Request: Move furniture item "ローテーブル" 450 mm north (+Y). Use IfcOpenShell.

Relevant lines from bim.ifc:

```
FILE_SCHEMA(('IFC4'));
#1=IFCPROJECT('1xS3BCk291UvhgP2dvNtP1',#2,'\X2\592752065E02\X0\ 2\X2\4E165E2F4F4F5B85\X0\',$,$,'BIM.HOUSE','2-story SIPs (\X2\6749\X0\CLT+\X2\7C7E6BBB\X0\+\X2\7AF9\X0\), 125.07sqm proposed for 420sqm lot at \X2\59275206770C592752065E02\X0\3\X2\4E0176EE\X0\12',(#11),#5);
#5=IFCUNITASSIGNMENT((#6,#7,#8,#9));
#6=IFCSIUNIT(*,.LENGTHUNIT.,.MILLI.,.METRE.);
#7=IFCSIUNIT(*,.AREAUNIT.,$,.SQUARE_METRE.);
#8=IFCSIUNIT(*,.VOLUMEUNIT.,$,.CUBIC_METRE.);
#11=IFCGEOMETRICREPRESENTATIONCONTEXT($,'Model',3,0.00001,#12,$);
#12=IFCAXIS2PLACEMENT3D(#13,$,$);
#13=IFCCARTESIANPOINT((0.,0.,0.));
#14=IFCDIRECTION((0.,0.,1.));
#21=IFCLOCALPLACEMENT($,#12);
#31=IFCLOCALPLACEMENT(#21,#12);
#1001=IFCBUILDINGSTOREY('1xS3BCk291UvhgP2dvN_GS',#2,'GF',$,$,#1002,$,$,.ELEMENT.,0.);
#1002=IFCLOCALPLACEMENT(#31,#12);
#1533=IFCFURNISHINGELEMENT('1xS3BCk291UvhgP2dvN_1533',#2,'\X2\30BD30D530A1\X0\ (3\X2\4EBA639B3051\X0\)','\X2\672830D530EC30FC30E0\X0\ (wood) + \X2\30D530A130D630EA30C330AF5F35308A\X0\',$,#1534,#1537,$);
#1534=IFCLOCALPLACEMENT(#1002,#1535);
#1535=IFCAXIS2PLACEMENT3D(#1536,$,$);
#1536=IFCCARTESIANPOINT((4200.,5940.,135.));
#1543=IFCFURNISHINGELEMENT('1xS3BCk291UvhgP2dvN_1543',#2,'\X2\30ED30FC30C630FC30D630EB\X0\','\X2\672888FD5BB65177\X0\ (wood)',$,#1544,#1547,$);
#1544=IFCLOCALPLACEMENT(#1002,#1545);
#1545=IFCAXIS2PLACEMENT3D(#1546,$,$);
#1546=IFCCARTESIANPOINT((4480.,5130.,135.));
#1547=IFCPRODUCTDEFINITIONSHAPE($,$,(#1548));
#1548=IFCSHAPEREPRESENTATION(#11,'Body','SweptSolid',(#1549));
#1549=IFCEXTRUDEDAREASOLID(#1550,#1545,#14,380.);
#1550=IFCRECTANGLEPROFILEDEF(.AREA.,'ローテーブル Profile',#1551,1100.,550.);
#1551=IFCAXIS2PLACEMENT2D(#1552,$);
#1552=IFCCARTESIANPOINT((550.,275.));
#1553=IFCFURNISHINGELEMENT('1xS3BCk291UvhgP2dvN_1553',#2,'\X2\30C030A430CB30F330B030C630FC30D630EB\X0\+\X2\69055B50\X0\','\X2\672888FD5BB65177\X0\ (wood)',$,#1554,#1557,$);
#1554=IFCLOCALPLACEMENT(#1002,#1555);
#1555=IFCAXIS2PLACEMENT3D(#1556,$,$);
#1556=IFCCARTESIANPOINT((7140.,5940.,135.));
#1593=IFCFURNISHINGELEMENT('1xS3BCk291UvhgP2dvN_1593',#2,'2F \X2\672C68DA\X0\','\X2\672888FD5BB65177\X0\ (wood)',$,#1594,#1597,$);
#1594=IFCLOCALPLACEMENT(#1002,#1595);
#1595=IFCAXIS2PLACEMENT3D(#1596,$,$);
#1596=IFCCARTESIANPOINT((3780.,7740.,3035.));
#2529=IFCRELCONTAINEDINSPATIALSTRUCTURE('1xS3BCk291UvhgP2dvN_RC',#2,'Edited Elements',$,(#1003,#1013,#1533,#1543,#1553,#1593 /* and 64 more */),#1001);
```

```python
import ifcopenshell
import ifcopenshell.api.geometry
import ifcopenshell.util.placement

model = ifcopenshell.open("bim.ifc")

item = model.by_guid("1xS3BCk291UvhgP2dvN_1543")
matrix = ifcopenshell.util.placement.get_local_placement(item.ObjectPlacement)
matrix[1, 3] += 450.0
ifcopenshell.api.geometry.edit_object_placement(model, product=item, matrix=matrix, is_si=False)

print(ifcopenshell.util.placement.get_local_placement(item.ObjectPlacement).round(3) + 0.0)

model.write("bim_edited.ifc")
```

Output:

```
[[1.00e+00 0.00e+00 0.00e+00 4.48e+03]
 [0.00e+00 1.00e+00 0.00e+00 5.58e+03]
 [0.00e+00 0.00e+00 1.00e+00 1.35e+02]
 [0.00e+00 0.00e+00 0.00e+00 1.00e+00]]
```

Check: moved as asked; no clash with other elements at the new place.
